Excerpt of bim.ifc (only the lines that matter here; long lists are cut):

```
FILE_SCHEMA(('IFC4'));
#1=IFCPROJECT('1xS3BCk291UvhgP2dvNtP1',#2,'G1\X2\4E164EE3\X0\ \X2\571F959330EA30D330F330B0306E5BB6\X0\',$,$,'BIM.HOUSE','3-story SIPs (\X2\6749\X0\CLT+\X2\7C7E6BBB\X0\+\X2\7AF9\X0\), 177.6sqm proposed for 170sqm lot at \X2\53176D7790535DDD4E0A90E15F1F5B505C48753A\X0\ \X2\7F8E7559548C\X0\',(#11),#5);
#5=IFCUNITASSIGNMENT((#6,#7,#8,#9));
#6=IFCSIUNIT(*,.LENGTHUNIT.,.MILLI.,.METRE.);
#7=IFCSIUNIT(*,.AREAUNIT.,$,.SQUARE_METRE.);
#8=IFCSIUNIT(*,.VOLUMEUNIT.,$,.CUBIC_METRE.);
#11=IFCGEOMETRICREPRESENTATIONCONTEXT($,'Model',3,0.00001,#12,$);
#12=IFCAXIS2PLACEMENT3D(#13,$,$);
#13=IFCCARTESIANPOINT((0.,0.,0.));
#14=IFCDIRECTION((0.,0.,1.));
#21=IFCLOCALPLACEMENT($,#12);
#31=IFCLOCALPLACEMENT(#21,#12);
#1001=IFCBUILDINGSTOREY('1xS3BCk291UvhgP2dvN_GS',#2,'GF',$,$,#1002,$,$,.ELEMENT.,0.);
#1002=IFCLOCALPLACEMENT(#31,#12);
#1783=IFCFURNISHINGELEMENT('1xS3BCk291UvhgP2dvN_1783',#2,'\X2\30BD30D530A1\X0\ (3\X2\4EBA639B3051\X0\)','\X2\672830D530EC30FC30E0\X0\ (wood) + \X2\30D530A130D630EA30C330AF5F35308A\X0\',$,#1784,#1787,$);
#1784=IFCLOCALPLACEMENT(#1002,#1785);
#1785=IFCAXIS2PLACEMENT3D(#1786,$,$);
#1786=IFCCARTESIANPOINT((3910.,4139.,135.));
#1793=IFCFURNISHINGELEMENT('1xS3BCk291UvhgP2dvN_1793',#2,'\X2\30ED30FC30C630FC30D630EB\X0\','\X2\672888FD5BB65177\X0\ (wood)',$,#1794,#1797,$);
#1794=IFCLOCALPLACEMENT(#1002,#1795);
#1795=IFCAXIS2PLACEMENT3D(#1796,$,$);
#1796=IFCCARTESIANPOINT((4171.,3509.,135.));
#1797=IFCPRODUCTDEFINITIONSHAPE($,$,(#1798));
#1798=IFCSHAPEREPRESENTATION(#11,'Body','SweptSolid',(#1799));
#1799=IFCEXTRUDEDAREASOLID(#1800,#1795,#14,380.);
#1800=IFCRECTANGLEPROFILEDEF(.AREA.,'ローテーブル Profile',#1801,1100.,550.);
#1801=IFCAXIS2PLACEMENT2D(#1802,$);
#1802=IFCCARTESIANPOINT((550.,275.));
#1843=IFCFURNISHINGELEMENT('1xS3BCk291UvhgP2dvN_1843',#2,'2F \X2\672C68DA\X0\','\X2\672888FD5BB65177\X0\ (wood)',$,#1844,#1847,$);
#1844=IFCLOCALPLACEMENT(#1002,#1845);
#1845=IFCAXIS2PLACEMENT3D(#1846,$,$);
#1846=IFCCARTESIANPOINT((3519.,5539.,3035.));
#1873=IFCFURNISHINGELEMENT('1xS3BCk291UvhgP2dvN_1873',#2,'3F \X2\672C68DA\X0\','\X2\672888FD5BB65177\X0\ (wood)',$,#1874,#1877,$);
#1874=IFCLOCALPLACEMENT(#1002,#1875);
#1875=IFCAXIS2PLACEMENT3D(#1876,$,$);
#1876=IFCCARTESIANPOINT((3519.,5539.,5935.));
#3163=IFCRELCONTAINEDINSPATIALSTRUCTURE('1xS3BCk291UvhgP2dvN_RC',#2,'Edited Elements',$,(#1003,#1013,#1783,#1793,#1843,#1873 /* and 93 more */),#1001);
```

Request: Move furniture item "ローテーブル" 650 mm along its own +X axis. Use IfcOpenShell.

```python
import ifcopenshell
import ifcopenshell.api.geometry
import ifcopenshell.util.placement

model = ifcopenshell.open("bim.ifc")

item = model.by_id(1793)
matrix = ifcopenshell.util.placement.get_local_placement(item.ObjectPlacement)
matrix[:3, 3] += matrix[:3, 0] * 650.0
ifcopenshell.api.geometry.edit_object_placement(model, product=item, matrix=matrix, is_si=False)

print(ifcopenshell.util.placement.get_local_placement(item.ObjectPlacement).round(3) + 0.0)

model.write("bim_updated.ifc")
```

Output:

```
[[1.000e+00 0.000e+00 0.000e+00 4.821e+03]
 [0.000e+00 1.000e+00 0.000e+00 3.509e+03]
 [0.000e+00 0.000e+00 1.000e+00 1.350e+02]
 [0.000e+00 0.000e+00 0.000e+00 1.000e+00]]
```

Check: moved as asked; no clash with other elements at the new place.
